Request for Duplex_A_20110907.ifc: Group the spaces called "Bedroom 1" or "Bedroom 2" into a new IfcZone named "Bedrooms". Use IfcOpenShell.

First a look at what the model holds.

```python
import ifcopenshell

model = ifcopenshell.open("Duplex_A_20110907.ifc")
print(model.schema)
seen = {}
for space in model.by_type("IfcSpace"):
    seen[space.LongName] = seen.get(space.LongName, 0) + 1
for name, count in sorted(seen.items(), key=str):
    print(count, "x", name)
print("zones:", [z.Name for z in model.by_type("IfcZone")][:20])
```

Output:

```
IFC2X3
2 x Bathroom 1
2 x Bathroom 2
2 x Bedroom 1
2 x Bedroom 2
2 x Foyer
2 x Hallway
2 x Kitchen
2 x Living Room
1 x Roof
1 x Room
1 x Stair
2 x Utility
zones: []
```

```python
import ifcopenshell
import ifcopenshell.api.group
import ifcopenshell.api.root

model = ifcopenshell.open("Duplex_A_20110907.ifc")

names = {"Bedroom 1", "Bedroom 2"}
spaces = [s for s in model.by_type("IfcSpace") if s.LongName in names]

zone = ifcopenshell.api.root.create_entity(model, ifc_class="IfcZone", name="Bedrooms")
ifcopenshell.api.group.assign_group(model, products=spaces, group=zone)
print(len(spaces), "spaces in", zone.Name)

model.write("Duplex_A_20110907_v2.ifc")
```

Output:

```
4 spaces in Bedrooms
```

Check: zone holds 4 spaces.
